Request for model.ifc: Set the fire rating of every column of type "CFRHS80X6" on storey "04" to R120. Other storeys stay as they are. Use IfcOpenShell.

First a look at what the model holds.

```python
import ifcopenshell
import ifcopenshell.util.element

model = ifcopenshell.open("model.ifc")
print(model.schema)
storey = next(s for s in model.by_type("IfcBuildingStorey") if s.Name == "04")
columns = [e for e in ifcopenshell.util.element.get_decomposition(storey) if e.is_a("IfcColumn")]
seen = {}
for e in columns:
    element_type = ifcopenshell.util.element.get_type(e)
    key = (element_type.Name if element_type != e and element_type else None, ifcopenshell.util.element.get_pset(e, "Pset_ColumnCommon", "FireRating"))
    seen[key] = seen.get(key, 0) + 1
for (name, value), count in sorted(seen.items(), key=str):
    print(count, "x", name, "|", value)
```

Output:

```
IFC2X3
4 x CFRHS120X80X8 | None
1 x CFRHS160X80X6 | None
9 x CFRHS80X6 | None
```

```python
import ifcopenshell
import ifcopenshell.api.pset
import ifcopenshell.util.element

model = ifcopenshell.open("model.ifc")

storey = next(s for s in model.by_type("IfcBuildingStorey") if s.Name == "04")
columns = [e for e in ifcopenshell.util.element.get_decomposition(storey) if e.is_a("IfcColumn")]

count = 0
for e in columns:
    element_type = ifcopenshell.util.element.get_type(e)
    if element_type in (None, e) or element_type.Name != "CFRHS80X6":
        continue
    # add_pset returns the element's existing set when there is one.
    pset = ifcopenshell.api.pset.add_pset(model, product=e, name="Pset_ColumnCommon")
    ifcopenshell.api.pset.edit_pset(model, pset=pset, properties={"FireRating": "R120"})
    count += 1

print(count, "columns updated")

model.write("model-out.ifc")
```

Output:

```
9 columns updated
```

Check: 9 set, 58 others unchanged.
